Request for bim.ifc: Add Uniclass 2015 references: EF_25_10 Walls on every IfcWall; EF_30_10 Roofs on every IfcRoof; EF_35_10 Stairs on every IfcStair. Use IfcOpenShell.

First a look at what the model holds.

```python
import ifcopenshell

model = ifcopenshell.open("bim.ifc")
print(model.schema)
print("classifications:", [c.Name for c in model.by_type("IfcClassification")])
for ifc_class in ("IfcDoor", "IfcRoof", "IfcStair", "IfcWall", "IfcWindow"):
    print(ifc_class, len(model.by_type(ifc_class)))
```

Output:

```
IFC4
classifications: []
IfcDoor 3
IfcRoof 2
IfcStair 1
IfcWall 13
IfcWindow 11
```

```python
import ifcopenshell
import ifcopenshell.api.classification

model = ifcopenshell.open("bim.ifc")

system = ifcopenshell.api.classification.add_classification(model, classification="Uniclass 2015")

codes = {
    "IfcWall": ("EF_25_10", "Walls"),
    "IfcRoof": ("EF_30_10", "Roofs"),
    "IfcStair": ("EF_35_10", "Stairs"),
}
for ifc_class, (code, name) in codes.items():
    products = model.by_type(ifc_class)
    ifcopenshell.api.classification.add_reference(
        model, products=products, classification=system, identification=code, name=name
    )
    print(code, len(products))

model.write("bim_rev.ifc")
```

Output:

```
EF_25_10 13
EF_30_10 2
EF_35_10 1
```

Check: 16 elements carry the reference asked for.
